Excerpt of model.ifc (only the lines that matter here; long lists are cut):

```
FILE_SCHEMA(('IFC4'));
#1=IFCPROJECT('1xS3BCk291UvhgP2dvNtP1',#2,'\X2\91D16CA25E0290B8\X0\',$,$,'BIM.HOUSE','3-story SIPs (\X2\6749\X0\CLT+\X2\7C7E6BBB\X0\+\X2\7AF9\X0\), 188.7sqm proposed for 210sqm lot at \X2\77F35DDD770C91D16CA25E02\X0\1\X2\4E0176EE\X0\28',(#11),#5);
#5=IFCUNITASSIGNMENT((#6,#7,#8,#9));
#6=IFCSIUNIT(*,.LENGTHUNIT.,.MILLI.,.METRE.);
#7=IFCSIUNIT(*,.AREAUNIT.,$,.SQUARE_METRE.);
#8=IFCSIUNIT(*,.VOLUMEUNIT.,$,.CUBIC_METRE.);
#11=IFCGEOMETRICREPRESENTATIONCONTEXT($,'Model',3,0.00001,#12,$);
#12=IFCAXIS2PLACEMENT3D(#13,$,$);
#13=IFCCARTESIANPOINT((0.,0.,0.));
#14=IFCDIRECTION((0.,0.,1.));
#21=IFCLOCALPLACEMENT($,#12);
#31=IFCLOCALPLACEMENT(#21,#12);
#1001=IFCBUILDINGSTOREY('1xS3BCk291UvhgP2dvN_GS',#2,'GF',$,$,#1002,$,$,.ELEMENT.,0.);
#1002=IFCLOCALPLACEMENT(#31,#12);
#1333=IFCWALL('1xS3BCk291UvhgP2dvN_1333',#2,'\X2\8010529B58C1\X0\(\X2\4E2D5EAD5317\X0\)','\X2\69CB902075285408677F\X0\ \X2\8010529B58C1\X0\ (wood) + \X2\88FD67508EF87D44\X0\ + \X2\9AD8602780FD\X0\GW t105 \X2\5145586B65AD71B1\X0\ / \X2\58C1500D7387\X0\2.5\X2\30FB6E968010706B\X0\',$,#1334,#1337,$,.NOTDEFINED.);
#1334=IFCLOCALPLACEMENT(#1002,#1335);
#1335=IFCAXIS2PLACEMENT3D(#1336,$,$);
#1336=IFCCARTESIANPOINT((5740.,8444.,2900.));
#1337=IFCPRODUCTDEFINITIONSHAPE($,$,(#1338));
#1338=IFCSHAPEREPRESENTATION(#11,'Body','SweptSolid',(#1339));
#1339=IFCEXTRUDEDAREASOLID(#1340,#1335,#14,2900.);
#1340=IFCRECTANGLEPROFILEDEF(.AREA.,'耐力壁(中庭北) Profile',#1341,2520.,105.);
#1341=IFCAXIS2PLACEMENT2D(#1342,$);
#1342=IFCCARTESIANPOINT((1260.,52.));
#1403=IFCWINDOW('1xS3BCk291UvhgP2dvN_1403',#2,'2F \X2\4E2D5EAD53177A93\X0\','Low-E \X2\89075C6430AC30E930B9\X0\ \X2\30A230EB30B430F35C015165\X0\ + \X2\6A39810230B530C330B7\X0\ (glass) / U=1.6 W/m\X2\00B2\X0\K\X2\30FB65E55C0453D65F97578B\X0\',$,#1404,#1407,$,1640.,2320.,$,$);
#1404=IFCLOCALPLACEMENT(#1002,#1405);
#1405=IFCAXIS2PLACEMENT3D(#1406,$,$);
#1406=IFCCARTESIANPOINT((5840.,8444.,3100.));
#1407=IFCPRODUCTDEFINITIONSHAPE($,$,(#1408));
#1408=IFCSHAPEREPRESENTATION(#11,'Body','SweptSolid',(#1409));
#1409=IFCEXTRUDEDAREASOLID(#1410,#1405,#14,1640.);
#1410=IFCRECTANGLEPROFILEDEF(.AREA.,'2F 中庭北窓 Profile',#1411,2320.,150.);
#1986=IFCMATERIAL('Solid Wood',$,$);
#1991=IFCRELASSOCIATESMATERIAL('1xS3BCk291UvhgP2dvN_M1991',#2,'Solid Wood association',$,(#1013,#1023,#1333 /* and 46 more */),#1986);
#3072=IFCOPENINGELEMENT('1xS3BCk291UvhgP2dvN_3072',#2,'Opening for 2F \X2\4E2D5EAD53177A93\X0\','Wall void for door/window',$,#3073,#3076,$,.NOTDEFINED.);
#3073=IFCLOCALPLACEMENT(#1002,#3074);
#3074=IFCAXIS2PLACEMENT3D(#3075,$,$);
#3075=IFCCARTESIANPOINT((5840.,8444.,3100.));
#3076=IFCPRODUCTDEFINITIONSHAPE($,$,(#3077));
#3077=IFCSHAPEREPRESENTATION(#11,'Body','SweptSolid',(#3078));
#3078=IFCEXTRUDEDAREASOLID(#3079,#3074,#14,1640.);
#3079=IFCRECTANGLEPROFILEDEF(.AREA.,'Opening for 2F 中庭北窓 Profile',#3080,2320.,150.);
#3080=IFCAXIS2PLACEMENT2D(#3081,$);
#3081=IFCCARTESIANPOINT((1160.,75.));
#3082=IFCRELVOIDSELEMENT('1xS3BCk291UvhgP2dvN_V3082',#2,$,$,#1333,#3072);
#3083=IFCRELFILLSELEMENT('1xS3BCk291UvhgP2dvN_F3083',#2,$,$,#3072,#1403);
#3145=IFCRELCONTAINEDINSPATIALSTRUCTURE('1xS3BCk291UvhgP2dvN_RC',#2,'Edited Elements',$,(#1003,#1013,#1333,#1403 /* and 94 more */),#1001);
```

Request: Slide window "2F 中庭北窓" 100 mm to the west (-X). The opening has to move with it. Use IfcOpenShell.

```python
import ifcopenshell
import ifcopenshell.api.geometry
import ifcopenshell.util.placement
import ifcopenshell.util.unit

model = ifcopenshell.open("model.ifc")
unit_scale = ifcopenshell.util.unit.calculate_unit_scale(model)

window = model.by_id(1403)
opening = window.FillsVoids[0].RelatingOpeningElement
wall = opening.VoidsElements[0].RelatingBuildingElement

wall_matrix = ifcopenshell.util.placement.get_local_placement(wall.ObjectPlacement)
shift = wall_matrix[:3, 0] * -0.1 / unit_scale
before = ifcopenshell.util.placement.get_local_placement(window.ObjectPlacement)[:3, 3].copy()

# The window is not placed relative to its opening, so move both.
for product in (opening, window):
    matrix = ifcopenshell.util.placement.get_local_placement(product.ObjectPlacement)
    matrix[:3, 3] += shift
    ifcopenshell.api.geometry.edit_object_placement(model, product=product, matrix=matrix, is_si=False)

after = ifcopenshell.util.placement.get_local_placement(window.ObjectPlacement)[:3, 3]
print("window moved by", (after - before).round(3) + 0.0)

model.write("model_updated.ifc")
```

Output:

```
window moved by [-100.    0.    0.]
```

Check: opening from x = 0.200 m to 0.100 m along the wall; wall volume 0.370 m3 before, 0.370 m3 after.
